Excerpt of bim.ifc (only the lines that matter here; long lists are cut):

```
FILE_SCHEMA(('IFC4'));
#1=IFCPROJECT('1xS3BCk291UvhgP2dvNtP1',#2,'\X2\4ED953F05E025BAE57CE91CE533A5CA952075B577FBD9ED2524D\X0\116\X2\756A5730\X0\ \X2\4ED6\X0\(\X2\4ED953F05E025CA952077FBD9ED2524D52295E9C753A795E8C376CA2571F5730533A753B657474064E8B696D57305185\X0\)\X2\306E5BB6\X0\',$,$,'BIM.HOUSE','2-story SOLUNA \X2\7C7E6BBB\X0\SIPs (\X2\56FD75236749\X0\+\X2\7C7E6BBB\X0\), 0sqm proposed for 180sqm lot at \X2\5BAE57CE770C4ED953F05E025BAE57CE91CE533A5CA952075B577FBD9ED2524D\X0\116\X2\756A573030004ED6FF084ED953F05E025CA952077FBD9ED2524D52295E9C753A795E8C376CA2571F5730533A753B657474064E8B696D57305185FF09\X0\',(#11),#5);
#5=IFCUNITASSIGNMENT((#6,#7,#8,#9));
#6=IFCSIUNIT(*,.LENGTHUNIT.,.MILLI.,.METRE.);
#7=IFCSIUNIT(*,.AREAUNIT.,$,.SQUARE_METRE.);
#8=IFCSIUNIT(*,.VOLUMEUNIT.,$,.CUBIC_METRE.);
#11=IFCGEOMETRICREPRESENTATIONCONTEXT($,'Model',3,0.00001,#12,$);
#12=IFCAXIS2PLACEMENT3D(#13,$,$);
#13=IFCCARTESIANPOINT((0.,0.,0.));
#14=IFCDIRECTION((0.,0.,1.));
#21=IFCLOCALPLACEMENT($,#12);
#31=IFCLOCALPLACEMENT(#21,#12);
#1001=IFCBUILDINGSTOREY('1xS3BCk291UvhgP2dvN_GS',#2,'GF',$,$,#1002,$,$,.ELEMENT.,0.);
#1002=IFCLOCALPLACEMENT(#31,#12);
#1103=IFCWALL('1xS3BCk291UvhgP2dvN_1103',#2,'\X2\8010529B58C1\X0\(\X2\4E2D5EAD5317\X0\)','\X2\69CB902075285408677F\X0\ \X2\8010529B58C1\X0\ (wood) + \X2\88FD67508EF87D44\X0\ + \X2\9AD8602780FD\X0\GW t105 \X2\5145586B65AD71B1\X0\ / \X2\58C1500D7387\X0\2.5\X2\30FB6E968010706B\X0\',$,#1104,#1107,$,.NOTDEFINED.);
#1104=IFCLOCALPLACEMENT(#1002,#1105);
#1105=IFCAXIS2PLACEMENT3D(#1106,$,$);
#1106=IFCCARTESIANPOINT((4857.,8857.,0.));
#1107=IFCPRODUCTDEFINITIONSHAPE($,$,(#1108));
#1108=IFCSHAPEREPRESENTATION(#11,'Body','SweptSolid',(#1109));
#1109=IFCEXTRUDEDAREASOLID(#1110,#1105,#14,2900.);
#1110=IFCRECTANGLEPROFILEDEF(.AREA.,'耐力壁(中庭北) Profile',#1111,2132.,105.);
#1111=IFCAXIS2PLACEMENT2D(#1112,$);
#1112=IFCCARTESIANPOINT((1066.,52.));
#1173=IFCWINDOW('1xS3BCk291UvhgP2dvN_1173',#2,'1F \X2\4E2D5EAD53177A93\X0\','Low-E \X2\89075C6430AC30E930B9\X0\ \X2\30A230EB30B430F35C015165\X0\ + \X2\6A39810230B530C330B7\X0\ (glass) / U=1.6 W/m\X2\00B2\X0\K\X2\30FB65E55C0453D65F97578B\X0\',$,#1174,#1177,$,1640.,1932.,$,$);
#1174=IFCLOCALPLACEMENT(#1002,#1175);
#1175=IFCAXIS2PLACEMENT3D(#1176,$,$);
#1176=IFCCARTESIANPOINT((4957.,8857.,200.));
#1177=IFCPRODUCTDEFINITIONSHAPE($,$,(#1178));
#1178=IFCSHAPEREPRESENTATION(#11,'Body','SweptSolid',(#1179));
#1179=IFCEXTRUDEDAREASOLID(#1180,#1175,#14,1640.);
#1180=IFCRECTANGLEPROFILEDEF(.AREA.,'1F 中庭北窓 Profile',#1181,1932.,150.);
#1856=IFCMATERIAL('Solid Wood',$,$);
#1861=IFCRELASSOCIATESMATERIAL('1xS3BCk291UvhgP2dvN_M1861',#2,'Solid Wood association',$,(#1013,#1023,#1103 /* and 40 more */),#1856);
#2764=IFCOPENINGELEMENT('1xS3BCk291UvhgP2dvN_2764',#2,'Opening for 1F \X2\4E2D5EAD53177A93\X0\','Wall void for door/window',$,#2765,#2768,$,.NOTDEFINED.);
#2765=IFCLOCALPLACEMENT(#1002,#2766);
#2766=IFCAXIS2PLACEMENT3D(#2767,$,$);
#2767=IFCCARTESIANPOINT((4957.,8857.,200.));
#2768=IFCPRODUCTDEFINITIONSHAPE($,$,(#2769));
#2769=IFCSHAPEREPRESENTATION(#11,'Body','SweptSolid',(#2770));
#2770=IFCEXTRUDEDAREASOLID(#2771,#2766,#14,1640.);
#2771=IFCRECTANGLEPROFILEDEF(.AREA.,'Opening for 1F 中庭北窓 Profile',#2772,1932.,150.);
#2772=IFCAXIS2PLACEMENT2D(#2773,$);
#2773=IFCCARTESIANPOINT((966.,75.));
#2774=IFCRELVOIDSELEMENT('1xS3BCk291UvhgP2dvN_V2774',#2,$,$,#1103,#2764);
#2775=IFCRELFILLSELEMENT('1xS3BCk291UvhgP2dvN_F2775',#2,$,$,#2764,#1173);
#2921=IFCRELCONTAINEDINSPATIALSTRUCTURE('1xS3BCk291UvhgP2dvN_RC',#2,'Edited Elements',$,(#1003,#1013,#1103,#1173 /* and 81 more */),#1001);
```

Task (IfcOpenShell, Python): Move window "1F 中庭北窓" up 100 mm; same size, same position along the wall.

```python
import numpy as np
import ifcopenshell
import ifcopenshell.api.geometry
import ifcopenshell.util.placement
import ifcopenshell.util.unit

model = ifcopenshell.open("bim.ifc")
unit_scale = ifcopenshell.util.unit.calculate_unit_scale(model)

window = model.by_guid("1xS3BCk291UvhgP2dvN_1173")
opening = window.FillsVoids[0].RelatingOpeningElement
dz = 100.0

shift = np.array([0.0, 0.0, dz])
# The window is not placed relative to its opening, so move both.
for product in (opening, window):
    matrix = ifcopenshell.util.placement.get_local_placement(product.ObjectPlacement)
    matrix[:3, 3] += shift
    ifcopenshell.api.geometry.edit_object_placement(model, product=product, matrix=matrix, is_si=False)

print(f"moved by {dz * unit_scale:+.3f} m")

model.write("bim-out.ifc")
```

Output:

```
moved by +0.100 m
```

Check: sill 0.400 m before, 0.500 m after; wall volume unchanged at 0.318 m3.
